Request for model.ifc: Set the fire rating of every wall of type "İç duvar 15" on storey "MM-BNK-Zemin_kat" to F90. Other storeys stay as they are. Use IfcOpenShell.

First a look at what the model holds.

```python
import ifcopenshell
import ifcopenshell.util.element

model = ifcopenshell.open("model.ifc")
print(model.schema)
storey = next(s for s in model.by_type("IfcBuildingStorey") if s.Name == "MM-BNK-Zemin_kat")
walls = [e for e in ifcopenshell.util.element.get_decomposition(storey) if e.is_a("IfcWall")]
seen = {}
for e in walls:
    element_type = ifcopenshell.util.element.get_type(e)
    key = (element_type.Name if element_type != e and element_type else None, ifcopenshell.util.element.get_pset(e, "Pset_WallCommon", "FireRating"))
    seen[key] = seen.get(key, 0) + 1
for (name, value), count in sorted(seen.items(), key=str):
    print(count, "x", name, "|", value)
```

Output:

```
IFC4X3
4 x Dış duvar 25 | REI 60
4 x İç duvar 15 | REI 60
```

```python
import ifcopenshell
import ifcopenshell.api.pset
import ifcopenshell.util.element

model = ifcopenshell.open("model.ifc")

storey = next(s for s in model.by_type("IfcBuildingStorey") if s.Name == "MM-BNK-Zemin_kat")
walls = [e for e in ifcopenshell.util.element.get_decomposition(storey) if e.is_a("IfcWall")]

count = 0
for e in walls:
    element_type = ifcopenshell.util.element.get_type(e)
    if element_type in (None, e) or element_type.Name != "İç duvar 15":
        continue
    # add_pset returns the element's existing set when there is one.
    pset = ifcopenshell.api.pset.add_pset(model, product=e, name="Pset_WallCommon")
    ifcopenshell.api.pset.edit_pset(model, pset=pset, properties={"FireRating": "F90"})
    count += 1

print(count, "walls updated")

model.write("model-out.ifc")
```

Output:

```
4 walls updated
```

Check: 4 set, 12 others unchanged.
